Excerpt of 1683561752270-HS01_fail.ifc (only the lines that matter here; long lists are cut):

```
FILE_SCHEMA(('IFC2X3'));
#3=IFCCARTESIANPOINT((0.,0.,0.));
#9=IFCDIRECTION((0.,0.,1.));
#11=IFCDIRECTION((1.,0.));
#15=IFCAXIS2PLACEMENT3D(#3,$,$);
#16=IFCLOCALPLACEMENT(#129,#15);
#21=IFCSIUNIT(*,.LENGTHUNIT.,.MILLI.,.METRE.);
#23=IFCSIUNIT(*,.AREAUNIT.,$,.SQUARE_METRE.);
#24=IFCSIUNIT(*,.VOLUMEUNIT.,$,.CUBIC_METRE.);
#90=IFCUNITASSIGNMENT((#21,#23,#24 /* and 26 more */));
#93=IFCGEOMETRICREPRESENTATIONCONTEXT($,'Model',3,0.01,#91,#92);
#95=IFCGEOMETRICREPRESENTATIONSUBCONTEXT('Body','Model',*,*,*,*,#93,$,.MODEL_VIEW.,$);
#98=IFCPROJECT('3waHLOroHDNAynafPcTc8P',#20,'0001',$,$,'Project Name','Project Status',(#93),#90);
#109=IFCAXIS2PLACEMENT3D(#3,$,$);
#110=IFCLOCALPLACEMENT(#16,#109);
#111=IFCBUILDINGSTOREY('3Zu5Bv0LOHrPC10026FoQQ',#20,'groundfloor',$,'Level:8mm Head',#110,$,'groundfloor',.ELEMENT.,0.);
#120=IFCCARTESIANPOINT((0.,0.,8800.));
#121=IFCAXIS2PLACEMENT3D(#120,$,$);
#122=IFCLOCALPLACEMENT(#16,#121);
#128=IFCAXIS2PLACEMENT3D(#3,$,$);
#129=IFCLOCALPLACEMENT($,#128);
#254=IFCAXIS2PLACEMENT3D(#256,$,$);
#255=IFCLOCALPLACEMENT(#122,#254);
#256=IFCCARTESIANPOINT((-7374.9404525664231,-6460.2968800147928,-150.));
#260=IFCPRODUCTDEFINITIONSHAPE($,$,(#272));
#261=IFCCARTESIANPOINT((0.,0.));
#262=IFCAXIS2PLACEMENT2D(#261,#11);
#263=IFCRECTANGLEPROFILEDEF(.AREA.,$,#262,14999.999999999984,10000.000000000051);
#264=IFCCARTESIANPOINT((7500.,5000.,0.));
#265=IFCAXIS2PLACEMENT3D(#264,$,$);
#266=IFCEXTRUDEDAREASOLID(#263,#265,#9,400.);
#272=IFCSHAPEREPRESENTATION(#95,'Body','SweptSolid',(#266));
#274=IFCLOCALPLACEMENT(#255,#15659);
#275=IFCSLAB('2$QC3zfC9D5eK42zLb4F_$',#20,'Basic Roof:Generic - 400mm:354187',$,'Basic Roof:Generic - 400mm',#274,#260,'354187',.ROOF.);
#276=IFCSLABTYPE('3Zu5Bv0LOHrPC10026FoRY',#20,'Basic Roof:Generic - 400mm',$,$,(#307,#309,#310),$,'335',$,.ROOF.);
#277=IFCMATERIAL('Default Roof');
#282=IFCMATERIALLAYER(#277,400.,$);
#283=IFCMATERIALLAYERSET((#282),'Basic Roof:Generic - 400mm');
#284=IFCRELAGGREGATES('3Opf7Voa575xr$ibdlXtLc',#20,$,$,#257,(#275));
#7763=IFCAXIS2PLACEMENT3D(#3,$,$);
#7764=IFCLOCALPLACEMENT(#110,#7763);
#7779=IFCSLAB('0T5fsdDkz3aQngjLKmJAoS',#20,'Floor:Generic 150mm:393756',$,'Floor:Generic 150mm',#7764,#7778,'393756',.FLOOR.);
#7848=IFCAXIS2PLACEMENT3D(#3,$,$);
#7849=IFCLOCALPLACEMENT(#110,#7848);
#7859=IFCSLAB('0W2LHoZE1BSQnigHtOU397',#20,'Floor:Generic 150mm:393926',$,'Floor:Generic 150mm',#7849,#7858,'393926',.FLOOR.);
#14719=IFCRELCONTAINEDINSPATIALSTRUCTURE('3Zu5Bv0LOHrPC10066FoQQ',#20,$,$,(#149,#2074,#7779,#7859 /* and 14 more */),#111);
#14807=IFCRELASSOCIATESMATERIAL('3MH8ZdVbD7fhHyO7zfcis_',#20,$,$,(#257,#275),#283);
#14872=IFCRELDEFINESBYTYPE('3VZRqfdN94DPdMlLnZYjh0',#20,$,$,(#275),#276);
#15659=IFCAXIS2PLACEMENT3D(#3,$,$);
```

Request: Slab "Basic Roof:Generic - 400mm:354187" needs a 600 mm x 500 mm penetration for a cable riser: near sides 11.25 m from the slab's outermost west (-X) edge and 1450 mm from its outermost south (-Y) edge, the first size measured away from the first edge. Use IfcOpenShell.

```python
import numpy as np
import ifcopenshell
import ifcopenshell.api.feature
import ifcopenshell.api.geometry
import ifcopenshell.api.root
import ifcopenshell.geom
import ifcopenshell.util.placement
import ifcopenshell.util.representation
import ifcopenshell.util.shape
import ifcopenshell.util.unit

model = ifcopenshell.open("1683561752270-HS01_fail.ifc")
unit_scale = ifcopenshell.util.unit.calculate_unit_scale(model)
settings = ifcopenshell.geom.settings()


def volume(element):
    """Net volume in cubic metres, openings subtracted."""
    shape = ifcopenshell.geom.create_shape(settings, element)
    return ifcopenshell.util.shape.get_volume(shape.geometry)


slab = model.by_guid("2$QC3zfC9D5eK42zLb4F_$")
before = volume(slab)

# Extent in the slab's own axes, in metres. The edges named are its -X and -Y sides.
slab_shape = ifcopenshell.geom.create_shape(settings, slab)
vertices = ifcopenshell.util.shape.get_vertices(slab_shape.geometry)
x_min, y_min, bottom = vertices.min(axis=0)
top = vertices[:, 2].max()

opening = ifcopenshell.api.root.create_entity(model, ifc_class="IfcOpeningElement", name="Cable riser opening")
context = ifcopenshell.util.representation.get_context(model, "Model", "Body", "MODEL_VIEW")
width, depth = 0.6, 0.5
outline = [(0.0, 0.0), (width, 0.0), (width, depth), (0.0, depth), (0.0, 0.0)]
# Overshoot both faces by 50 mm so the cut is clean.
shape = ifcopenshell.api.geometry.add_slab_representation(
    model, context=context, depth=top - bottom + 0.1, polyline=outline
)
ifcopenshell.api.geometry.assign_representation(model, product=opening, representation=shape)

matrix = ifcopenshell.util.placement.get_local_placement(slab.ObjectPlacement)
matrix[:, 3] = matrix @ np.append(np.array([x_min + 11.25, y_min + 1.45, bottom - 0.05]) / unit_scale, 1.0)
ifcopenshell.api.geometry.edit_object_placement(model, product=opening, matrix=matrix, is_si=False)
ifcopenshell.api.feature.add_feature(model, feature=opening, element=slab)

after = volume(slab)

print(f"slab volume {before:.3f} -> {after:.3f} m3")

model.write("1683561752270-HS01_fail-out.ifc")
```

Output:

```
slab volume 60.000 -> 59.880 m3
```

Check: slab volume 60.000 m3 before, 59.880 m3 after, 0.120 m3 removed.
